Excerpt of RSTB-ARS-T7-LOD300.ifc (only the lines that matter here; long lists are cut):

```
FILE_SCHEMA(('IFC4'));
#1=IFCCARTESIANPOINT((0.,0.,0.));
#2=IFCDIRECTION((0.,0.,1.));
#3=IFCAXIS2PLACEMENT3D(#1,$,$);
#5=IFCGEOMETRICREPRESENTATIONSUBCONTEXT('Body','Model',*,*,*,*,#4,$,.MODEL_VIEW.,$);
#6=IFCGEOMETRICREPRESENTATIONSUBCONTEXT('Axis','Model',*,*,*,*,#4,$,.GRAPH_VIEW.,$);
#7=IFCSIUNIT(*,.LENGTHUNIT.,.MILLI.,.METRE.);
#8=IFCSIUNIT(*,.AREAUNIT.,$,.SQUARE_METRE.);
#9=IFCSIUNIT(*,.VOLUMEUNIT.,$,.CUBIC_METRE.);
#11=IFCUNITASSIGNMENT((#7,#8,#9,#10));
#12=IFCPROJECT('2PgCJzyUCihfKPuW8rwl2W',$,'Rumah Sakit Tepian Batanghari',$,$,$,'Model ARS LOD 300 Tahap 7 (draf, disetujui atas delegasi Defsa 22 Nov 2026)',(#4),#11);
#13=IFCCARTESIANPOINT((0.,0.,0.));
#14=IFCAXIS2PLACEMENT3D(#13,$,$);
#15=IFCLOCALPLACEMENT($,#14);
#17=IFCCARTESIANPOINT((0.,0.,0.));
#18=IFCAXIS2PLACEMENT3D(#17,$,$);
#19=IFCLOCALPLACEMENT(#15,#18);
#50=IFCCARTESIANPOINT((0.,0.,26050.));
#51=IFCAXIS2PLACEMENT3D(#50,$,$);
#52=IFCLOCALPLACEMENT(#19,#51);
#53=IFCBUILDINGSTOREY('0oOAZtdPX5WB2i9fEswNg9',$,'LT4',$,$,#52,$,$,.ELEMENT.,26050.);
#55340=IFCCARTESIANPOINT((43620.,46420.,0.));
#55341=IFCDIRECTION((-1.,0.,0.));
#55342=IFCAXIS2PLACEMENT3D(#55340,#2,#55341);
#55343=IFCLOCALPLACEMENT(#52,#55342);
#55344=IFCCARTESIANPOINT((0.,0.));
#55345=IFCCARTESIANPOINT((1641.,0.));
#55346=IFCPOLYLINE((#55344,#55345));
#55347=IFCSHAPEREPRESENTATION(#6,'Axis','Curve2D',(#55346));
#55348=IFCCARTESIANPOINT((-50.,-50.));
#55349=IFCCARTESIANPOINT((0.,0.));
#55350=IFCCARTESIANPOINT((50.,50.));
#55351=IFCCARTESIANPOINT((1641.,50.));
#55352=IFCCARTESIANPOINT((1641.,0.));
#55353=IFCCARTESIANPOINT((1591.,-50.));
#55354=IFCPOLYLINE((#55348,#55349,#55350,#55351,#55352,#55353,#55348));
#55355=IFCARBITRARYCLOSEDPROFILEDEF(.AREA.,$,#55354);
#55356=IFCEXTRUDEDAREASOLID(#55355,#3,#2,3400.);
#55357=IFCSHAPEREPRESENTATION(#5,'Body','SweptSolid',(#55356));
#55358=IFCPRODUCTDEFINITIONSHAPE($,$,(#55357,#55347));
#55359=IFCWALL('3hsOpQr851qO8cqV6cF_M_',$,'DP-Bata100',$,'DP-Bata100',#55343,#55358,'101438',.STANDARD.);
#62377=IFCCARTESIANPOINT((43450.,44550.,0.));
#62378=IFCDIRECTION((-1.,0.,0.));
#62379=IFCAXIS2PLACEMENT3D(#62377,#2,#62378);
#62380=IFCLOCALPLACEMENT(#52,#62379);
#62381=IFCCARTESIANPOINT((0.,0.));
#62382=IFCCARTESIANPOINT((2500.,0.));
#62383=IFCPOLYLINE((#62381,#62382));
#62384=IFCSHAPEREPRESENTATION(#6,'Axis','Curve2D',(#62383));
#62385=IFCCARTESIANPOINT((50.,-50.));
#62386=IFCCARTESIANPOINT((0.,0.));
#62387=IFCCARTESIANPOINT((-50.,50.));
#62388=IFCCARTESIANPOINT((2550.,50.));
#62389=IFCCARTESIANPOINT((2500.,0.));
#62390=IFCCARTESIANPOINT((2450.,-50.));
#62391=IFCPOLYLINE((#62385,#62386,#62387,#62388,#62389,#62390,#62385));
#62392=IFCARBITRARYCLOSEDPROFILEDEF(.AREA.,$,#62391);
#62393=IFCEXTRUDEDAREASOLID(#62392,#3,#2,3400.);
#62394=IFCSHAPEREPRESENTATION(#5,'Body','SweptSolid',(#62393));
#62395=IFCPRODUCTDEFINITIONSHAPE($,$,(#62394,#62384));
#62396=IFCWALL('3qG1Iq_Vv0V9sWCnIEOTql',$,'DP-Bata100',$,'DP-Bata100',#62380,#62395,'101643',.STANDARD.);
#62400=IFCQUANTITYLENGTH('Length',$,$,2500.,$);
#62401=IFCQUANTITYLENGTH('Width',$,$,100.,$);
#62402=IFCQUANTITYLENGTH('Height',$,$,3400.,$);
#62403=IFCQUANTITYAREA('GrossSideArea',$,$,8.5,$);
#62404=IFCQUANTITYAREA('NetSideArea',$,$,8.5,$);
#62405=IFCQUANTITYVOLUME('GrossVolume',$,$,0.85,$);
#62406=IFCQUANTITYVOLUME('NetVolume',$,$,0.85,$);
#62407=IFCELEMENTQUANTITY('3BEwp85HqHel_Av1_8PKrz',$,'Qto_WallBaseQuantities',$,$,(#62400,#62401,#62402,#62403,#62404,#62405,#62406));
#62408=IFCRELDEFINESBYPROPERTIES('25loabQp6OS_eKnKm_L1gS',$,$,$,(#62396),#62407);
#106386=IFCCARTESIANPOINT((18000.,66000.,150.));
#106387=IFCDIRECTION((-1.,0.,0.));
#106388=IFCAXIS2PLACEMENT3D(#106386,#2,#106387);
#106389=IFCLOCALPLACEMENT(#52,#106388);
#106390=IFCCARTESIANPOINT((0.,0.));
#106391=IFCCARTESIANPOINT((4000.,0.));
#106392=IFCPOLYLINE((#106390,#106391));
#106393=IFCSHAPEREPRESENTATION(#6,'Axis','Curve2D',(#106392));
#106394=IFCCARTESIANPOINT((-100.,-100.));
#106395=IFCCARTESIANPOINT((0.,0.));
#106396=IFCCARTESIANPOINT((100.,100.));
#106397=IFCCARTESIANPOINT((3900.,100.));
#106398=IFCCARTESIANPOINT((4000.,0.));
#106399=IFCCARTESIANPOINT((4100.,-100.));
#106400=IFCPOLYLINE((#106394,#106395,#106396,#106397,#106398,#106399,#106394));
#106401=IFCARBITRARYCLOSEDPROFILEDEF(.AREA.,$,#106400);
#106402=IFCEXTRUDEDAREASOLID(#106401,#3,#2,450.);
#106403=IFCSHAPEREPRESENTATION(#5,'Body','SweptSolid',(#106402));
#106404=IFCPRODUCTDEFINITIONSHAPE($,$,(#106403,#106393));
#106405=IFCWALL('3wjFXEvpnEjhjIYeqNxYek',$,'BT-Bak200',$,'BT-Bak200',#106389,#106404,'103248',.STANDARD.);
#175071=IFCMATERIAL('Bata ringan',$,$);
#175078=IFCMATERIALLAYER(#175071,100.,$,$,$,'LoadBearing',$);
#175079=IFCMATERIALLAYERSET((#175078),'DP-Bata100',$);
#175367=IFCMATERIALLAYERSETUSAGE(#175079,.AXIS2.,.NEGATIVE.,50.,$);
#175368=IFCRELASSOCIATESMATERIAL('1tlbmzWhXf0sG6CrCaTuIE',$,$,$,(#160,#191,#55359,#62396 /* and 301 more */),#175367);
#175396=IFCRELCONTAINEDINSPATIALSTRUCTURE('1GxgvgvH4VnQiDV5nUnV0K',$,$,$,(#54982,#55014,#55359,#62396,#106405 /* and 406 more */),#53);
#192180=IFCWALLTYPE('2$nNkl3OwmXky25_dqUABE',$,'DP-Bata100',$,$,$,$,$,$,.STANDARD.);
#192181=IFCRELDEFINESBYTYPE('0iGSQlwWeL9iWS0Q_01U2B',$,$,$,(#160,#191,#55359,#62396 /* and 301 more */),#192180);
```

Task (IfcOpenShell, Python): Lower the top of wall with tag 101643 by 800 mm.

```python
import ifcopenshell
import ifcopenshell.api.pset
import ifcopenshell.geom
import ifcopenshell.util.element
import ifcopenshell.util.representation
import ifcopenshell.util.shape
import ifcopenshell.util.unit

model = ifcopenshell.open("RSTB-ARS-T7-LOD300.ifc")
unit_scale = ifcopenshell.util.unit.calculate_unit_scale(model)
area_scale = ifcopenshell.util.unit.calculate_unit_scale(model, "AREAUNIT")
volume_scale = ifcopenshell.util.unit.calculate_unit_scale(model, "VOLUMEUNIT")
settings = ifcopenshell.geom.settings()


def volume(element):
    """Net volume in cubic metres, openings subtracted."""
    shape = ifcopenshell.geom.create_shape(settings, element)
    return ifcopenshell.util.shape.get_volume(shape.geometry)


wall = model.by_id(62396)
before = volume(wall)

body = ifcopenshell.util.representation.get_representation(wall, "Model", "Body")
solid = body.Items[0]
old_height = solid.Depth
solid.Depth -= 0.8 / unit_scale
after = volume(wall)
thickness = 0.1  # wall thickness in metres

# Update the stored height, areas and volumes.
qto = model.by_id(ifcopenshell.util.element.get_pset(wall, "Qto_WallBaseQuantities", should_inherit=False)["id"])
ifcopenshell.api.pset.edit_qto(model, qto=qto, properties={
    "Height": solid.Depth,
    "GrossSideArea": ifcopenshell.util.element.get_pset(wall, "Qto_WallBaseQuantities", "GrossSideArea") * solid.Depth / old_height,
    "NetSideArea": after / thickness / area_scale,
    "GrossVolume": ifcopenshell.util.element.get_pset(wall, "Qto_WallBaseQuantities", "GrossVolume") * solid.Depth / old_height,
    "NetVolume": after / volume_scale,
})

print(f"height {old_height:g} -> {solid.Depth:g}, volume {before:.3f} -> {after:.3f} m3")

model.write("RSTB-ARS-T7-LOD300_v2.ifc")
```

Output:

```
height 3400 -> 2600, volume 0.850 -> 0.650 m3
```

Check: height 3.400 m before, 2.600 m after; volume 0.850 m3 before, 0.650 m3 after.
